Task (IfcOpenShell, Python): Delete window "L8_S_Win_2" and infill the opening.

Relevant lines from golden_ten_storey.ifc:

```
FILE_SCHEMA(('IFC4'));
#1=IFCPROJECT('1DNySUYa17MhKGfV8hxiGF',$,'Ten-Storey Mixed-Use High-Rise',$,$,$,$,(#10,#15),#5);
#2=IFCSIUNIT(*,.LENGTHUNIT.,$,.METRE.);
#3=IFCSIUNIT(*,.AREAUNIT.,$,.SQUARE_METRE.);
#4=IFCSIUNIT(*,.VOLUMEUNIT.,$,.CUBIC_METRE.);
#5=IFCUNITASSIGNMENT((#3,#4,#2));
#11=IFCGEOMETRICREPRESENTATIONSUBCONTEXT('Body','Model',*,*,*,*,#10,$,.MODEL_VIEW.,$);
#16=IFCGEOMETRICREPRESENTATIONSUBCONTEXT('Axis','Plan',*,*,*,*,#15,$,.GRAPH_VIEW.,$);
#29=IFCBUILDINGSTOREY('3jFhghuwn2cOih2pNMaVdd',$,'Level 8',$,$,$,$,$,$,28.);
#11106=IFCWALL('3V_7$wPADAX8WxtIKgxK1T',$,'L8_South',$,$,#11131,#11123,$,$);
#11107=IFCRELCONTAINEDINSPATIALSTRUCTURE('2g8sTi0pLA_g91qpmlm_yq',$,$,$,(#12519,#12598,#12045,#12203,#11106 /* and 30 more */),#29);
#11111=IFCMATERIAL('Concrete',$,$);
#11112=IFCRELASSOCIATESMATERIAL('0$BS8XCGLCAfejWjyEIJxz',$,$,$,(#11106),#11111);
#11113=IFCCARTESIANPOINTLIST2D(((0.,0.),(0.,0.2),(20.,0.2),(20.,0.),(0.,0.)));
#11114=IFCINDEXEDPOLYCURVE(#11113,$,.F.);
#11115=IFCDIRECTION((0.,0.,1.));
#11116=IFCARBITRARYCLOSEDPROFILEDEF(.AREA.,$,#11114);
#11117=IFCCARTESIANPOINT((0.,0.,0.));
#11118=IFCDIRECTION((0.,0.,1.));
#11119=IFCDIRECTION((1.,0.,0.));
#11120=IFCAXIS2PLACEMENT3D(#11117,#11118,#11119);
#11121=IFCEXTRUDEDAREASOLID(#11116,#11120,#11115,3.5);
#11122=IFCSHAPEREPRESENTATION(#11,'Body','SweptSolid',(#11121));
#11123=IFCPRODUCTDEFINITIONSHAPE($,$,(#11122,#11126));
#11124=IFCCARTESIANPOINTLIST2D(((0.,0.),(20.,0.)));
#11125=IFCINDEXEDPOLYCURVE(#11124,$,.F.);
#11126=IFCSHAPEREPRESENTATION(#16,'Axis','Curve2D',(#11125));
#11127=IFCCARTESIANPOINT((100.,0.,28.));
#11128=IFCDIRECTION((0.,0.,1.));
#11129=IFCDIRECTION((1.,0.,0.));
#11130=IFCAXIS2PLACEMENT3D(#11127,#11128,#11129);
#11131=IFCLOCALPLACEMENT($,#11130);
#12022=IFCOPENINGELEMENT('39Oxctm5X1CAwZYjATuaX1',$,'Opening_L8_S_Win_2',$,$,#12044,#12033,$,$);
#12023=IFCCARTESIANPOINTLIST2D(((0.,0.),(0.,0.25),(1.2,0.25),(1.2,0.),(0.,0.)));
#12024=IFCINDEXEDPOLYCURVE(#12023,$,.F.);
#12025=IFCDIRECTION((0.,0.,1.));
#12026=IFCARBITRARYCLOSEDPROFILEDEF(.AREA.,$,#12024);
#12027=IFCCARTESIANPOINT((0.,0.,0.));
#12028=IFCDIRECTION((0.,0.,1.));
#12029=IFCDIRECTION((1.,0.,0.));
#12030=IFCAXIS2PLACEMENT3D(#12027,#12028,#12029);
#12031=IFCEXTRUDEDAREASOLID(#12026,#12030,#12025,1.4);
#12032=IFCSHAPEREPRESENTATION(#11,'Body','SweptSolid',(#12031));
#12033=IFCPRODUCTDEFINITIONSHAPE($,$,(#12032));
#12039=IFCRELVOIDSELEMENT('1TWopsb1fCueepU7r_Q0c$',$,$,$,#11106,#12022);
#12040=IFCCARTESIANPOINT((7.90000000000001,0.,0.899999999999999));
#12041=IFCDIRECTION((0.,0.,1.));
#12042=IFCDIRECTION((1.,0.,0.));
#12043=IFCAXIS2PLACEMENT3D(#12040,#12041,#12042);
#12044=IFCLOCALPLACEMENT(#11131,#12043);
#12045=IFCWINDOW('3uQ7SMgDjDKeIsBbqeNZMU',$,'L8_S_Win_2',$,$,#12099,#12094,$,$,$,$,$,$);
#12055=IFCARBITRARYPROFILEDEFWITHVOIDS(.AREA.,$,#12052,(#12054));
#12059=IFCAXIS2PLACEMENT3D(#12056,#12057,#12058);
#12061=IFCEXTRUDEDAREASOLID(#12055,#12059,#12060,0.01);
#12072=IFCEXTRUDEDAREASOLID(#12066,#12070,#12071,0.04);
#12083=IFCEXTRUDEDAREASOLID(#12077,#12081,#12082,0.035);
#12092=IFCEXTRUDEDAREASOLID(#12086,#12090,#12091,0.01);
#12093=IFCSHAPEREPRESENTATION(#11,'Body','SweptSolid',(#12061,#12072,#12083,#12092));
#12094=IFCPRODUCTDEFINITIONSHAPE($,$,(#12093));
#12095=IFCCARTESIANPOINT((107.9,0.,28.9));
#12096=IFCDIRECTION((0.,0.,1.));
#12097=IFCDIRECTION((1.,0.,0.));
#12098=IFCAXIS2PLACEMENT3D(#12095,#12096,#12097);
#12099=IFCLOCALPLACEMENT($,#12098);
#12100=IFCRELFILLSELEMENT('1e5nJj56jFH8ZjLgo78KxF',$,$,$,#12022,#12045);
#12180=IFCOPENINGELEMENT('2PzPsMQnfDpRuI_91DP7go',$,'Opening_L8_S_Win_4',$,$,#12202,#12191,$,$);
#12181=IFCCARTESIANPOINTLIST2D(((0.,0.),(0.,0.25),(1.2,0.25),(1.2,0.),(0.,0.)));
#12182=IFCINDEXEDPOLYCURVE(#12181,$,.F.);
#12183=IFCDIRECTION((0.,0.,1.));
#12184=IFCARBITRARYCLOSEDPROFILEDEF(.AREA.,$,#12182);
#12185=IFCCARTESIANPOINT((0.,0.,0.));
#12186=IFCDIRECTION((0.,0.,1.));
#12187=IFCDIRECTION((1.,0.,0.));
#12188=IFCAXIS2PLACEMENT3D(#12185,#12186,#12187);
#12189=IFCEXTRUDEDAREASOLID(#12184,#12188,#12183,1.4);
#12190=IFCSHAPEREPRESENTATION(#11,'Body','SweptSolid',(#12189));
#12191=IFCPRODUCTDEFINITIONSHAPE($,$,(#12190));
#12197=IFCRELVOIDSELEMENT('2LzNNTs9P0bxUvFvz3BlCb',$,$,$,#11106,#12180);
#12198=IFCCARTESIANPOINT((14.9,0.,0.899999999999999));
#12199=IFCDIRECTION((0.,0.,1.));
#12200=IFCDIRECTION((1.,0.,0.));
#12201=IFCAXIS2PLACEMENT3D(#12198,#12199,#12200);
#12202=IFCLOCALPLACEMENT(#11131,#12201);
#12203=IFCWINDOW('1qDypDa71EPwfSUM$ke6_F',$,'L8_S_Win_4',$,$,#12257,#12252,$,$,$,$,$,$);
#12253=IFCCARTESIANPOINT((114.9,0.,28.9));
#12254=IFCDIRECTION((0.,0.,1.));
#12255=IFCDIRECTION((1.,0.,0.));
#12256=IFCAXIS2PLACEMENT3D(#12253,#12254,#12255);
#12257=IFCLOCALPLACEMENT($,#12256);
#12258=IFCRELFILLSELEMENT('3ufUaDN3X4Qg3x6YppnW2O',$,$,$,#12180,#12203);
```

```python
import ifcopenshell
import ifcopenshell.api.feature
import ifcopenshell.api.root
import ifcopenshell.geom
import ifcopenshell.util.shape

model = ifcopenshell.open("golden_ten_storey.ifc")
settings = ifcopenshell.geom.settings()


def volume(element):
    """Net volume in cubic metres, openings subtracted."""
    shape = ifcopenshell.geom.create_shape(settings, element)
    return ifcopenshell.util.shape.get_volume(shape.geometry)


window = model.by_guid("3uQ7SMgDjDKeIsBbqeNZMU")
opening = window.FillsVoids[0].RelatingOpeningElement
wall = opening.VoidsElements[0].RelatingBuildingElement
before = volume(wall)

ifcopenshell.api.root.remove_product(model, product=window)
ifcopenshell.api.feature.remove_feature(model, feature=opening)

after = volume(wall)

print(f"wall volume {before:.3f} -> {after:.3f} m3")

model.write("golden_ten_storey_edited.ifc")
```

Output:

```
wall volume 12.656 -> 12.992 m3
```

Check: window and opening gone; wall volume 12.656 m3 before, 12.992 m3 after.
